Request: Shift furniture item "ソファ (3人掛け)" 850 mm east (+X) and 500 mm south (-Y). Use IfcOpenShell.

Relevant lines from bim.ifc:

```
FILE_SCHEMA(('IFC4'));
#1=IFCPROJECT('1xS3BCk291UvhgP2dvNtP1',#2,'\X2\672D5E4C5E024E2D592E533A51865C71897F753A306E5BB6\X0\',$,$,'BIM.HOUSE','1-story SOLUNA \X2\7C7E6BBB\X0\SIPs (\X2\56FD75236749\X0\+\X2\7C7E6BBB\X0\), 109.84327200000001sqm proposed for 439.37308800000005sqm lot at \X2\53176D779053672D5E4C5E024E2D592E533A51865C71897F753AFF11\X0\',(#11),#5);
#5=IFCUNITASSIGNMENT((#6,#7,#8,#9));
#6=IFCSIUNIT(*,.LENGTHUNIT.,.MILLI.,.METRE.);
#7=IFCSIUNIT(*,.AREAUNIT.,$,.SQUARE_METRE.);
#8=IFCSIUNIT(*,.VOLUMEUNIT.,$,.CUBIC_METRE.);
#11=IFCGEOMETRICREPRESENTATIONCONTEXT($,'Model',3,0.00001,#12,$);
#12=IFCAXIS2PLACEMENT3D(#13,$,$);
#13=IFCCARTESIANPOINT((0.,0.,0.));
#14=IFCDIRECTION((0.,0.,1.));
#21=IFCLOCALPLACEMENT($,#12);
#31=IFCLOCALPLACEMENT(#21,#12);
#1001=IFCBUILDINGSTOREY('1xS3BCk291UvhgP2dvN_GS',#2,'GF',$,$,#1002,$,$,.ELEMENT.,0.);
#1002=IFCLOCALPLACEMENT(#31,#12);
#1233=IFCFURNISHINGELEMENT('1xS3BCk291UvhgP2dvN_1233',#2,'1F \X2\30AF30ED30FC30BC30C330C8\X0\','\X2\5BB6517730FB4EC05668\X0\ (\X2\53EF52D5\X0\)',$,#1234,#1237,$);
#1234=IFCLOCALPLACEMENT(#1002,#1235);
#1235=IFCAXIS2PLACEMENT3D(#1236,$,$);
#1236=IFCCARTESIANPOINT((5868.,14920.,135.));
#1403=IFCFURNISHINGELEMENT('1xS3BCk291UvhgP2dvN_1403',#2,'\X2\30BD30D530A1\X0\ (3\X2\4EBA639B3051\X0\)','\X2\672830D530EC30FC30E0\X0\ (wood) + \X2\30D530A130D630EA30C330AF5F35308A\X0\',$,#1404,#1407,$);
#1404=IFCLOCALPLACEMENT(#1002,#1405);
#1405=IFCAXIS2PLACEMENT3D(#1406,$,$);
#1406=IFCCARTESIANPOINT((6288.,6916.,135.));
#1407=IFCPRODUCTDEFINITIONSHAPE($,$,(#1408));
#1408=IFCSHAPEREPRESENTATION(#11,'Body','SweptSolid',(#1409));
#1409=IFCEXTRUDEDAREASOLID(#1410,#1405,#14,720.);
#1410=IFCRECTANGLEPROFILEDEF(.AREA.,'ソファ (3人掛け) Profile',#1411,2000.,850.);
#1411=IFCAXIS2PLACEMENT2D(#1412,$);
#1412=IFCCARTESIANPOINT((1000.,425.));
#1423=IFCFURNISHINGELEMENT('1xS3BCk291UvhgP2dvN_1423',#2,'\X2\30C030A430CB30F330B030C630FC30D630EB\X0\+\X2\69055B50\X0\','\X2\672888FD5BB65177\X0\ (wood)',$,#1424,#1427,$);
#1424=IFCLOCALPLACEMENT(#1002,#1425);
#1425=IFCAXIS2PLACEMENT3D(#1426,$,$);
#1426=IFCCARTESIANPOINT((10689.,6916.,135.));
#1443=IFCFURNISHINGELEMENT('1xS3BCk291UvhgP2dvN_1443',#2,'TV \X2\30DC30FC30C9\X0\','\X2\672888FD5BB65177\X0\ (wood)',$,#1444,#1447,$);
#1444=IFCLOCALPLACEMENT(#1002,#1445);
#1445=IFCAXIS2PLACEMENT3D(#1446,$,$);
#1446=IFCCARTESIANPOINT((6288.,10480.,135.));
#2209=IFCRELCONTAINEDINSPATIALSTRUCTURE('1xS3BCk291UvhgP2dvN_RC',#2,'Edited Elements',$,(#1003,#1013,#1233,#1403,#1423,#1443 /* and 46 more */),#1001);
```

```python
import ifcopenshell
import ifcopenshell.api.geometry
import ifcopenshell.util.placement
import ifcopenshell.util.unit

model = ifcopenshell.open("bim.ifc")
unit_scale = ifcopenshell.util.unit.calculate_unit_scale(model)

item = model.by_id(1403)
matrix = ifcopenshell.util.placement.get_local_placement(item.ObjectPlacement)
matrix[0, 3] += 0.85 / unit_scale
matrix[1, 3] -= 0.5 / unit_scale
ifcopenshell.api.geometry.edit_object_placement(model, product=item, matrix=matrix, is_si=False)

print(ifcopenshell.util.placement.get_local_placement(item.ObjectPlacement).round(3) + 0.0)

model.write("bim_rev.ifc")
```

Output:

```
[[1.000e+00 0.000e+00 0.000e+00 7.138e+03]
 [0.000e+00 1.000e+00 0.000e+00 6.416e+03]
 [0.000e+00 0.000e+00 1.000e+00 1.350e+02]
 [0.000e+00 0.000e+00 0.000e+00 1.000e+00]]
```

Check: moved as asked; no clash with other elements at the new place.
